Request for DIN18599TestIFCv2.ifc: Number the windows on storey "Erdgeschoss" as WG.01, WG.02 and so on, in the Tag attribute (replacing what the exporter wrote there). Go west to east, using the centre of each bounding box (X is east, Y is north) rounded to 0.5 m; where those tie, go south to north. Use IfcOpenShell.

First a look at what the model holds.

```python
import ifcopenshell
import ifcopenshell.util.element
import ifcopenshell.util.placement

model = ifcopenshell.open("DIN18599TestIFCv2.ifc")
print(model.schema)
storey = next(s for s in model.by_type("IfcBuildingStorey") if s.Name == "Erdgeschoss")
windows = [e for e in ifcopenshell.util.element.get_decomposition(storey) if e.is_a("IfcWindow")]
for e in sorted(windows, key=lambda e: e.id()):
    origin = ifcopenshell.util.placement.get_local_placement(e.ObjectPlacement)[:3, 3]
    print(e.id(), e.Tag, e.Name, origin.round(2) + 0.0, sep=" | ")
```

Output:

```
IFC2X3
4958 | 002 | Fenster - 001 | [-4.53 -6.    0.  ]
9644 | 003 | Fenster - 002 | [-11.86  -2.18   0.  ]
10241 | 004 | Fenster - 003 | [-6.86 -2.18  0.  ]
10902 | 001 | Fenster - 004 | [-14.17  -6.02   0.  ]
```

```python
import ifcopenshell
import ifcopenshell.geom
import ifcopenshell.util.element
import ifcopenshell.util.shape

model = ifcopenshell.open("DIN18599TestIFCv2.ifc")
settings = ifcopenshell.geom.settings()
settings.set("use-world-coords", True)


def centre(element):
    shape = ifcopenshell.geom.create_shape(settings, element)
    return ifcopenshell.util.shape.get_bbox_centroid(shape.geometry)


storey = next(s for s in model.by_type("IfcBuildingStorey") if s.Name == "Erdgeschoss")
windows = [e for e in ifcopenshell.util.element.get_decomposition(storey) if e.is_a("IfcWindow")]

# Insertion points can sit at a corner or the storey origin, so sort by the geometry (in metres).
centres = {e: centre(e) for e in windows}
windows.sort(key=lambda e: (round(centres[e][0] / 0.5), centres[e][1]))

for i, e in enumerate(windows, start=1):
    number = f"WG.{i:02d}"
    e.Tag = number
    print(e.id(), number)

model.write("DIN18599TestIFCv2_updated.ifc")
```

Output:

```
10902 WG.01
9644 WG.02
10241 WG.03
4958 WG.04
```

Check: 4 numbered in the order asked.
